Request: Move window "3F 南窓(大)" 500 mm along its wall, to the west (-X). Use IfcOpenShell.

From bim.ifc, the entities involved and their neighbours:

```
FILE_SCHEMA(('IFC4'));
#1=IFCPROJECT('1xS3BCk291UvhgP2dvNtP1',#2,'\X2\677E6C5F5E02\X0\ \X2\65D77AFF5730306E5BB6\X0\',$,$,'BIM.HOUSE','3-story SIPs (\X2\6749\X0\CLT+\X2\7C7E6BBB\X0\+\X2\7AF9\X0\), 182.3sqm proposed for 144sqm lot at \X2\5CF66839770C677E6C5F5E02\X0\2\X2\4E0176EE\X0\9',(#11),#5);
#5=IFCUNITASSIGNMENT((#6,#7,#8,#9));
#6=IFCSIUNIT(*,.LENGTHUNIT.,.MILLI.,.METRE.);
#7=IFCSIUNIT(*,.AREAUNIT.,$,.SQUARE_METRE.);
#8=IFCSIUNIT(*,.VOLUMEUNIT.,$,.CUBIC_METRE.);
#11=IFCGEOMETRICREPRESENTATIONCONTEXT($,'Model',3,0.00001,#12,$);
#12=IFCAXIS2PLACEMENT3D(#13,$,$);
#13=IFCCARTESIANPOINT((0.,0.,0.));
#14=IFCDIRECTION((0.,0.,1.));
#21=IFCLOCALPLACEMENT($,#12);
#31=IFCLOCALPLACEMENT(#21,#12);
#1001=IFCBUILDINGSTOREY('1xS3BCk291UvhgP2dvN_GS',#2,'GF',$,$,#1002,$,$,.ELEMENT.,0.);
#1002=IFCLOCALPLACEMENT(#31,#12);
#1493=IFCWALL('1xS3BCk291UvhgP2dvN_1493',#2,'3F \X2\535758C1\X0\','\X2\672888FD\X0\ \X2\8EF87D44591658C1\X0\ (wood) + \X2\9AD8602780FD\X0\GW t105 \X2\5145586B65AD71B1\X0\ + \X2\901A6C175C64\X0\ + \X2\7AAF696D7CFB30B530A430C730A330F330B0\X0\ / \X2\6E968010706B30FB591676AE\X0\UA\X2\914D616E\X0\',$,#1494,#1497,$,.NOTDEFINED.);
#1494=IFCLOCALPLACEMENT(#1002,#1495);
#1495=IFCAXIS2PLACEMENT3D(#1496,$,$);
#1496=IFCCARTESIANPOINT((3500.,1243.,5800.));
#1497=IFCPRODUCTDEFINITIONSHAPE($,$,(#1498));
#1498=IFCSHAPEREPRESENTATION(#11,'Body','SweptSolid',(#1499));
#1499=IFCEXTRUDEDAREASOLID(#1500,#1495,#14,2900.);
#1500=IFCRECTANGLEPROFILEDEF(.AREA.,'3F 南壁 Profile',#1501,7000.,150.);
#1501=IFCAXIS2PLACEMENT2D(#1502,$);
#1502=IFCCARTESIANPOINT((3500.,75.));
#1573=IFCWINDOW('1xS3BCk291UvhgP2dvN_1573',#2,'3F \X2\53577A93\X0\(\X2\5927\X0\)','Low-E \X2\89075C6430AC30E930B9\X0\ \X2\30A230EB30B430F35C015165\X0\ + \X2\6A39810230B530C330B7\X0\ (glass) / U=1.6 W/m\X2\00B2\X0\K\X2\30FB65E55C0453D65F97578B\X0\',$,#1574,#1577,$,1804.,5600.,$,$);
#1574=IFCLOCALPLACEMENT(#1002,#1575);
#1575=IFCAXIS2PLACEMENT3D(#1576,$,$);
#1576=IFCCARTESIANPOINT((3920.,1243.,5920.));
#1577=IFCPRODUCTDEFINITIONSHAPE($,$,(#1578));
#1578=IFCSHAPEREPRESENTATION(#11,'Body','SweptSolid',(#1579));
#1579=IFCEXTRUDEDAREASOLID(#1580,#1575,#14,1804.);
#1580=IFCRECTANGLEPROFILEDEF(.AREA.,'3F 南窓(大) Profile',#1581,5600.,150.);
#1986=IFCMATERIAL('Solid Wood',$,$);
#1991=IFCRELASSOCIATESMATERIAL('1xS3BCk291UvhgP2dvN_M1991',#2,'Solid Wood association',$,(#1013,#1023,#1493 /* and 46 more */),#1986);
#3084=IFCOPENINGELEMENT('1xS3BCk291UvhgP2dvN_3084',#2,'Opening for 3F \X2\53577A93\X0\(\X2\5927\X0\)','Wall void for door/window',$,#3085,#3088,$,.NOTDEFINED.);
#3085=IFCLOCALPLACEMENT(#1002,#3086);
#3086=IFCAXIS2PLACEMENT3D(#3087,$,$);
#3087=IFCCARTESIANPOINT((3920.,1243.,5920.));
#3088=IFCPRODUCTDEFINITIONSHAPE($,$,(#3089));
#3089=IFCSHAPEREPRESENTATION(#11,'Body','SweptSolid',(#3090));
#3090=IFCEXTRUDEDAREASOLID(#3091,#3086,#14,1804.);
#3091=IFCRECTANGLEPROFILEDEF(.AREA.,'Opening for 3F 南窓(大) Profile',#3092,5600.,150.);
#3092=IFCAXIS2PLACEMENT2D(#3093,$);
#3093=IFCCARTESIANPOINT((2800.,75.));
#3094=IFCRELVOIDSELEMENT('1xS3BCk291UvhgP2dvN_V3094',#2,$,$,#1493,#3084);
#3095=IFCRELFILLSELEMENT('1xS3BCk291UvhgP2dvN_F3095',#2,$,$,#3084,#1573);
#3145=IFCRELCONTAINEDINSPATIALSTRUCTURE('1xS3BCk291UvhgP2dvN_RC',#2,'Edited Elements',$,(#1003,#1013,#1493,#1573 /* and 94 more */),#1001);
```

```python
import ifcopenshell
import ifcopenshell.api.geometry
import ifcopenshell.util.placement

model = ifcopenshell.open("bim.ifc")

window = model.by_guid("1xS3BCk291UvhgP2dvN_1573")
opening = window.FillsVoids[0].RelatingOpeningElement
wall = opening.VoidsElements[0].RelatingBuildingElement

wall_matrix = ifcopenshell.util.placement.get_local_placement(wall.ObjectPlacement)
shift = wall_matrix[:3, 0] * -500.0
before = ifcopenshell.util.placement.get_local_placement(window.ObjectPlacement)[:3, 3].copy()

# The window is not placed relative to its opening, so move both.
for product in (opening, window):
    matrix = ifcopenshell.util.placement.get_local_placement(product.ObjectPlacement)
    matrix[:3, 3] += shift
    ifcopenshell.api.geometry.edit_object_placement(model, product=product, matrix=matrix, is_si=False)

after = ifcopenshell.util.placement.get_local_placement(window.ObjectPlacement)[:3, 3]
print("window moved by", (after - before).round(3) + 0.0)

model.write("bim_v2.ifc")
```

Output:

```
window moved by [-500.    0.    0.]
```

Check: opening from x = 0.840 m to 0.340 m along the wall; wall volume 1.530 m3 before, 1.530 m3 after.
